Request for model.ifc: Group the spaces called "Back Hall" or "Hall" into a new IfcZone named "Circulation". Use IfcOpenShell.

First a look at what the model holds.

```python
import ifcopenshell

model = ifcopenshell.open("model.ifc")
print(model.schema)
seen = {}
for space in model.by_type("IfcSpace"):
    seen[space.LongName] = seen.get(space.LongName, 0) + 1
for name, count in sorted(seen.items(), key=str):
    print(count, "x", name)
print("zones:", [z.Name for z in model.by_type("IfcZone")][:20])
```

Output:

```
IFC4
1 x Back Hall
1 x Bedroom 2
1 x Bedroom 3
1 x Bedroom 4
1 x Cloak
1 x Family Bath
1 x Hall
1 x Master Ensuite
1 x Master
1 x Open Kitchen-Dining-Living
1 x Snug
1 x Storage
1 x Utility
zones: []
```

```python
import ifcopenshell
import ifcopenshell.api.group
import ifcopenshell.api.root

model = ifcopenshell.open("model.ifc")

names = {"Back Hall", "Hall"}
spaces = [s for s in model.by_type("IfcSpace") if s.LongName in names]

zone = ifcopenshell.api.root.create_entity(model, ifc_class="IfcZone", name="Circulation")
ifcopenshell.api.group.assign_group(model, products=spaces, group=zone)
print(len(spaces), "spaces in", zone.Name)

model.write("model_rev.ifc")
```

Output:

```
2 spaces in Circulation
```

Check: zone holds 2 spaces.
